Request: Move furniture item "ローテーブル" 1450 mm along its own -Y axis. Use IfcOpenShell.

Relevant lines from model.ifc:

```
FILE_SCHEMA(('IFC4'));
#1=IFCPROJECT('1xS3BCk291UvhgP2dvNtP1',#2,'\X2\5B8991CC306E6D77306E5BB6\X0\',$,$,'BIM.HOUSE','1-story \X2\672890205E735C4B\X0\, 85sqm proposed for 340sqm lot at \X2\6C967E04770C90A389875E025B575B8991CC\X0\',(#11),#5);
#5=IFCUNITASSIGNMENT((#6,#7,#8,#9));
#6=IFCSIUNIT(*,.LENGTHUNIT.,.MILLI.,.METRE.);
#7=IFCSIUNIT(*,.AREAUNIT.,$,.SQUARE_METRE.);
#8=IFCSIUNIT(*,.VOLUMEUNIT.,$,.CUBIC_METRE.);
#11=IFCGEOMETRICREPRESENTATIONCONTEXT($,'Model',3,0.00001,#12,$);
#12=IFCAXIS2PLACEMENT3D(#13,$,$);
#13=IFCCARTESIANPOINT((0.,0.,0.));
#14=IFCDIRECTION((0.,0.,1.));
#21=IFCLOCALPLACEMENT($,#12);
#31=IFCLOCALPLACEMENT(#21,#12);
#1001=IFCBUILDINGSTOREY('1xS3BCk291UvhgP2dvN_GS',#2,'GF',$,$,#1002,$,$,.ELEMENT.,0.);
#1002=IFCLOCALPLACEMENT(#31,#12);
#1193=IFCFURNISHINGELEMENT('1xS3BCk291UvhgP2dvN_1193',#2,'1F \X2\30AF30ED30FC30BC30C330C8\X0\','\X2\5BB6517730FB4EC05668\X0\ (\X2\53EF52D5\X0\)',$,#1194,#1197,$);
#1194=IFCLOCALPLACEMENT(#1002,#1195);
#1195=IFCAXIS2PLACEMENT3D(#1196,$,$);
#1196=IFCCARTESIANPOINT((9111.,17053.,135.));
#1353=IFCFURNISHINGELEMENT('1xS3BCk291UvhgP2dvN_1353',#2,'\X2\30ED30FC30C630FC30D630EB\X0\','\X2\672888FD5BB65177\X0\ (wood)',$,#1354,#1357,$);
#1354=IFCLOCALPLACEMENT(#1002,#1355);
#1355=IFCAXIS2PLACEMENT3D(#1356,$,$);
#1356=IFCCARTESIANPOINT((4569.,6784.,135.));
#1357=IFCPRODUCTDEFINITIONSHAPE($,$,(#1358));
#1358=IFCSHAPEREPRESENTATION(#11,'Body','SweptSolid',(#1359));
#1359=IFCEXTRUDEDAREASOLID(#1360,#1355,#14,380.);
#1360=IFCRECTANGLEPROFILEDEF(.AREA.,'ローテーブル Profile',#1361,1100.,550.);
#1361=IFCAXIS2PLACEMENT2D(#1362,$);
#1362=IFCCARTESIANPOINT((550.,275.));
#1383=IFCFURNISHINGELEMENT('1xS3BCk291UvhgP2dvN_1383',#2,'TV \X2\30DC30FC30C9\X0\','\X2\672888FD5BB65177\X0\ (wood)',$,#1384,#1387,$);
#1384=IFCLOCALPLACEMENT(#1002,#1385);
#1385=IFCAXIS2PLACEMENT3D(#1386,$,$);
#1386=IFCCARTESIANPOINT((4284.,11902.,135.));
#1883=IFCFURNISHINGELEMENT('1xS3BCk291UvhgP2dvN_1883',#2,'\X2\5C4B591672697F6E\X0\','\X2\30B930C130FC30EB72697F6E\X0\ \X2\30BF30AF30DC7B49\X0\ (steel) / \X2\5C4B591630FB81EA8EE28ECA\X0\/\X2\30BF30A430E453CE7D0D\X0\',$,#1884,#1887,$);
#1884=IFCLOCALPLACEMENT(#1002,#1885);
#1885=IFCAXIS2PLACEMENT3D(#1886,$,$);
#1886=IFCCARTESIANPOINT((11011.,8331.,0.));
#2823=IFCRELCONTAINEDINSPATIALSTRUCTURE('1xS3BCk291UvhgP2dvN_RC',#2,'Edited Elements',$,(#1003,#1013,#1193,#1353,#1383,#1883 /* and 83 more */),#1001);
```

```python
import ifcopenshell
import ifcopenshell.api.geometry
import ifcopenshell.util.placement
import ifcopenshell.util.unit

model = ifcopenshell.open("model.ifc")
unit_scale = ifcopenshell.util.unit.calculate_unit_scale(model)

item = model.by_guid("1xS3BCk291UvhgP2dvN_1353")
matrix = ifcopenshell.util.placement.get_local_placement(item.ObjectPlacement)
matrix[:3, 3] -= matrix[:3, 1] * 1.45 / unit_scale
ifcopenshell.api.geometry.edit_object_placement(model, product=item, matrix=matrix, is_si=False)

print(ifcopenshell.util.placement.get_local_placement(item.ObjectPlacement).round(3) + 0.0)

model.write("model_edited.ifc")
```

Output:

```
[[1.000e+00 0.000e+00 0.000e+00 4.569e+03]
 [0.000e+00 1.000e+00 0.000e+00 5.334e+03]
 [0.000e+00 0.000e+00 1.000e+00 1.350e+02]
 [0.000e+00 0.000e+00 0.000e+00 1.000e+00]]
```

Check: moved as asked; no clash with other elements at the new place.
